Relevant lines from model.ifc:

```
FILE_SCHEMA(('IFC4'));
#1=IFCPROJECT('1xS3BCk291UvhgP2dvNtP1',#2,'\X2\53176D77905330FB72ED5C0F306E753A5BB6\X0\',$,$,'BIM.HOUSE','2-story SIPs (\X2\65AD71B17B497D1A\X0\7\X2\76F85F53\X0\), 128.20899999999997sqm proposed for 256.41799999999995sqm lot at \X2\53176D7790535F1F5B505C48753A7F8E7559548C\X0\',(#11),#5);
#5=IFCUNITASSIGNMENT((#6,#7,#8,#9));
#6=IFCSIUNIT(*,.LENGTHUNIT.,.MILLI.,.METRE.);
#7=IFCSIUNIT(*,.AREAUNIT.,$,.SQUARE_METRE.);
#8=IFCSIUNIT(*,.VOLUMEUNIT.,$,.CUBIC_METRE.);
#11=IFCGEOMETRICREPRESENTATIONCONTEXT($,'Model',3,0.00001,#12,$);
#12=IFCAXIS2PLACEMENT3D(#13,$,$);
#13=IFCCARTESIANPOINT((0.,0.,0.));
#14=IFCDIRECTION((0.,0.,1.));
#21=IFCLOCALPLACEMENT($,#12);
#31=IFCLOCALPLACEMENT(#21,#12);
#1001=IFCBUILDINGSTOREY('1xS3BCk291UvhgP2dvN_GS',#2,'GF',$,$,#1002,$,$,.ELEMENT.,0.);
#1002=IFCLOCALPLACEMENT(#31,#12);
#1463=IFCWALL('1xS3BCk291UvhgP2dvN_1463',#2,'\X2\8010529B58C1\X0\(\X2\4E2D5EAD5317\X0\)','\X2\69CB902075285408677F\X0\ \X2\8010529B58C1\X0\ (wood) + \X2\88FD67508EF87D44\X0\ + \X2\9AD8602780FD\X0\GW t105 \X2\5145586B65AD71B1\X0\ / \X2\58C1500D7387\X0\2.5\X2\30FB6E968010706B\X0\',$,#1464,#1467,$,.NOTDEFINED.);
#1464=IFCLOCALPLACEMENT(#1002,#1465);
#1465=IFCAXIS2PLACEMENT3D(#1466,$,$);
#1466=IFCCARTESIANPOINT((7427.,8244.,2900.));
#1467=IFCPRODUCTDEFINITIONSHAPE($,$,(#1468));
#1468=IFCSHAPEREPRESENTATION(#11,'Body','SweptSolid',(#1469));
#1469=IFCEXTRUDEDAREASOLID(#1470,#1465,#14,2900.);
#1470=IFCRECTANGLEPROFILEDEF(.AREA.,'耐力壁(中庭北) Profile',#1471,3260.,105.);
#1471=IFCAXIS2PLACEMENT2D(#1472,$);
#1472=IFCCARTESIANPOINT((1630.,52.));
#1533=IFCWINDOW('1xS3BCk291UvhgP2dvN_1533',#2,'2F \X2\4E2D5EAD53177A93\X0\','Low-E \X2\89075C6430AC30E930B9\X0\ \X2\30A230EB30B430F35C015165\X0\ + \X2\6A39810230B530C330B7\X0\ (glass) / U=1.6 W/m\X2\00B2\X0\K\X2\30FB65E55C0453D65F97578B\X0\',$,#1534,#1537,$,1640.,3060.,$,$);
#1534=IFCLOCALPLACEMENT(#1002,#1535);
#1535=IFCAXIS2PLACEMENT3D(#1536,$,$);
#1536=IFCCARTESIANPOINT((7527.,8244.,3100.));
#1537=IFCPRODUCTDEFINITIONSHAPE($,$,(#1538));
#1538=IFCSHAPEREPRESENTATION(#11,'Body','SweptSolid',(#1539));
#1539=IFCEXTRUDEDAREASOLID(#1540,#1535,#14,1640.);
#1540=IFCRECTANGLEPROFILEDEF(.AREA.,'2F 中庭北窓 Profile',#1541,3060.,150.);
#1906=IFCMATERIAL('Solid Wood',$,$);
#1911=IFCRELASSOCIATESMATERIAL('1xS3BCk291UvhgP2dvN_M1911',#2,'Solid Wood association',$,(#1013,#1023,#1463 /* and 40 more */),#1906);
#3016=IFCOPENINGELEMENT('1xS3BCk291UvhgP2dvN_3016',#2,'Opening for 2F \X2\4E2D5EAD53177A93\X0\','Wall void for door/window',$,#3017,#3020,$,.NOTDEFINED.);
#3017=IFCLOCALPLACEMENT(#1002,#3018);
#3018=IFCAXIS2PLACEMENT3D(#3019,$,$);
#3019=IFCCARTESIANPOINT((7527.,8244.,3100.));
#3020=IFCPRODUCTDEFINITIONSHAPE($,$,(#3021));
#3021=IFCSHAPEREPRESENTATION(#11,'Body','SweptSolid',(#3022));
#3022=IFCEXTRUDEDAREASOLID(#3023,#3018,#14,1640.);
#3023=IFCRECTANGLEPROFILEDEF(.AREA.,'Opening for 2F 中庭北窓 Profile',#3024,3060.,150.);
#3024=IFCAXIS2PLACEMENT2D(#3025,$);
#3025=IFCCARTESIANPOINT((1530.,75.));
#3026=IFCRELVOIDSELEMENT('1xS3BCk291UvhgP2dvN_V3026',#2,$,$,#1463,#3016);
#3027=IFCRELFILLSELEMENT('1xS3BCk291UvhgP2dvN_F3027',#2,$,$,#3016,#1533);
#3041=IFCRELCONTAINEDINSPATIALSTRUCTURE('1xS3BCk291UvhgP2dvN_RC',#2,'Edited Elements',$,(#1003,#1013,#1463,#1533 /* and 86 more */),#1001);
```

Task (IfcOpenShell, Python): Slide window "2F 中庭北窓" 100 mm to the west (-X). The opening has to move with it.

```python
import ifcopenshell
import ifcopenshell.api.geometry
import ifcopenshell.util.placement
import ifcopenshell.util.unit

model = ifcopenshell.open("model.ifc")
unit_scale = ifcopenshell.util.unit.calculate_unit_scale(model)

window = model.by_id(1533)
opening = window.FillsVoids[0].RelatingOpeningElement
wall = opening.VoidsElements[0].RelatingBuildingElement

wall_matrix = ifcopenshell.util.placement.get_local_placement(wall.ObjectPlacement)
shift = wall_matrix[:3, 0] * -0.1 / unit_scale
before = ifcopenshell.util.placement.get_local_placement(window.ObjectPlacement)[:3, 3].copy()

# The window is not placed relative to its opening, so move both.
for product in (opening, window):
    matrix = ifcopenshell.util.placement.get_local_placement(product.ObjectPlacement)
    matrix[:3, 3] += shift
    ifcopenshell.api.geometry.edit_object_placement(model, product=product, matrix=matrix, is_si=False)

after = ifcopenshell.util.placement.get_local_placement(window.ObjectPlacement)[:3, 3]
print("window moved by", (after - before).round(3) + 0.0)

model.write("model_rev.ifc")
```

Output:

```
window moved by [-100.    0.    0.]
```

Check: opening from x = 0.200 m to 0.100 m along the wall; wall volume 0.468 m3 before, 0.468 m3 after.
